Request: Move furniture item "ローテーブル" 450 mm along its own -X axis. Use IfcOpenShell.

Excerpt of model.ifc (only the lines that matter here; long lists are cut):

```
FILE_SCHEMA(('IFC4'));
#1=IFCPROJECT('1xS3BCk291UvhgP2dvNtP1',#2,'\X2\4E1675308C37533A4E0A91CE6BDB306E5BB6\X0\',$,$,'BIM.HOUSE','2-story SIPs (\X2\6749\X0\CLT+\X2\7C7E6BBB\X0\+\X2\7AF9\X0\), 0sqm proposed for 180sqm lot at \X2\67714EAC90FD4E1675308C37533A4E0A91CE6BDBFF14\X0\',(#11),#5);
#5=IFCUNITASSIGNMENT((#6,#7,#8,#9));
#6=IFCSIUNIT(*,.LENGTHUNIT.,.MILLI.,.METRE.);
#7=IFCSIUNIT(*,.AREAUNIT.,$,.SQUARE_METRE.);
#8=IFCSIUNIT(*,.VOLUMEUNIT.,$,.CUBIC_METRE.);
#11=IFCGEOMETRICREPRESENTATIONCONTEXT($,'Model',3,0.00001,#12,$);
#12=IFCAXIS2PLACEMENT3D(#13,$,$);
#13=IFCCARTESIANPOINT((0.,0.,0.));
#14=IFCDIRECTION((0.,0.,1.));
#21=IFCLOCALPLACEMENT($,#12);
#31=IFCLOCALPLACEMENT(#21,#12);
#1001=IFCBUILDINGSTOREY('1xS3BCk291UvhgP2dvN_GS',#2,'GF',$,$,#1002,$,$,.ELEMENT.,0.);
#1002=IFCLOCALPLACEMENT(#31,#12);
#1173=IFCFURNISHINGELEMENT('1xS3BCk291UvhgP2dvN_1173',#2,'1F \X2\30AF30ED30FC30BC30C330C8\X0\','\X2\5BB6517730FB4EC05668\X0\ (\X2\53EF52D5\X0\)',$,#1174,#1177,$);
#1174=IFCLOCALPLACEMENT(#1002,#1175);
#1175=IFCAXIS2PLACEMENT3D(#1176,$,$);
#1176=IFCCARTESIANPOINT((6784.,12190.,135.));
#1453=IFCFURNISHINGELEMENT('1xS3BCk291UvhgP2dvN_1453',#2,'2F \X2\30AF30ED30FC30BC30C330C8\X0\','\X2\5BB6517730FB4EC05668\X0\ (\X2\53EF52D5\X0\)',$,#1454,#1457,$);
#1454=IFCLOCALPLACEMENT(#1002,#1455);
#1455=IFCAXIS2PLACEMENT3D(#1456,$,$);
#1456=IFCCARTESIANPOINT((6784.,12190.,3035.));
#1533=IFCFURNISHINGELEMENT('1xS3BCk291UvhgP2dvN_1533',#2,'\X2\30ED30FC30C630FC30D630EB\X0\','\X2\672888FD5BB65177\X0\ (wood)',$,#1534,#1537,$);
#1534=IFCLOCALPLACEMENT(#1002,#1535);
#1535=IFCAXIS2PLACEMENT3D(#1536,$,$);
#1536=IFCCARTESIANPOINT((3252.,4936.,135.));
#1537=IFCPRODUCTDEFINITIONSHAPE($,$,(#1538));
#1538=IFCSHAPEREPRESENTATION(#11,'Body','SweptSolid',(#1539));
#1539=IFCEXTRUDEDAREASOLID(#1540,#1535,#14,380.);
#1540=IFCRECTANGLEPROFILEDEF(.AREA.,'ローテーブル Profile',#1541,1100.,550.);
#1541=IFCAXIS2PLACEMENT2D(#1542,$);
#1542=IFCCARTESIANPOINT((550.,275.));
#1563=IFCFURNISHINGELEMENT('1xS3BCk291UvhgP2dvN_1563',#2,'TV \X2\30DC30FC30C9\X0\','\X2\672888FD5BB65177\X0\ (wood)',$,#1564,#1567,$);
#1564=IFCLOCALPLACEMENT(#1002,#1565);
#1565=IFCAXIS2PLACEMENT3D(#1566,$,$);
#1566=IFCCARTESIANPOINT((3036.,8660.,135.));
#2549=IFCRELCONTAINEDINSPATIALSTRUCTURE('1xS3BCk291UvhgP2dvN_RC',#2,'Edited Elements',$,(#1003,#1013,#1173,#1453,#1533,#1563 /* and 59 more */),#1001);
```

```python
import ifcopenshell
import ifcopenshell.api.geometry
import ifcopenshell.util.placement

model = ifcopenshell.open("model.ifc")

item = model.by_guid("1xS3BCk291UvhgP2dvN_1533")
matrix = ifcopenshell.util.placement.get_local_placement(item.ObjectPlacement)
matrix[:3, 3] -= matrix[:3, 0] * 450.0
ifcopenshell.api.geometry.edit_object_placement(model, product=item, matrix=matrix, is_si=False)

print(ifcopenshell.util.placement.get_local_placement(item.ObjectPlacement).round(3) + 0.0)

model.write("model_rev.ifc")
```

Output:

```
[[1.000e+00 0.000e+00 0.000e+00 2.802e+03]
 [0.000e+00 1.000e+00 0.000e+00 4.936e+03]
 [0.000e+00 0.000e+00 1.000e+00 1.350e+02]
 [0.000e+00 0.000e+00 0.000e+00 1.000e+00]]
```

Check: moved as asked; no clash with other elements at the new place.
